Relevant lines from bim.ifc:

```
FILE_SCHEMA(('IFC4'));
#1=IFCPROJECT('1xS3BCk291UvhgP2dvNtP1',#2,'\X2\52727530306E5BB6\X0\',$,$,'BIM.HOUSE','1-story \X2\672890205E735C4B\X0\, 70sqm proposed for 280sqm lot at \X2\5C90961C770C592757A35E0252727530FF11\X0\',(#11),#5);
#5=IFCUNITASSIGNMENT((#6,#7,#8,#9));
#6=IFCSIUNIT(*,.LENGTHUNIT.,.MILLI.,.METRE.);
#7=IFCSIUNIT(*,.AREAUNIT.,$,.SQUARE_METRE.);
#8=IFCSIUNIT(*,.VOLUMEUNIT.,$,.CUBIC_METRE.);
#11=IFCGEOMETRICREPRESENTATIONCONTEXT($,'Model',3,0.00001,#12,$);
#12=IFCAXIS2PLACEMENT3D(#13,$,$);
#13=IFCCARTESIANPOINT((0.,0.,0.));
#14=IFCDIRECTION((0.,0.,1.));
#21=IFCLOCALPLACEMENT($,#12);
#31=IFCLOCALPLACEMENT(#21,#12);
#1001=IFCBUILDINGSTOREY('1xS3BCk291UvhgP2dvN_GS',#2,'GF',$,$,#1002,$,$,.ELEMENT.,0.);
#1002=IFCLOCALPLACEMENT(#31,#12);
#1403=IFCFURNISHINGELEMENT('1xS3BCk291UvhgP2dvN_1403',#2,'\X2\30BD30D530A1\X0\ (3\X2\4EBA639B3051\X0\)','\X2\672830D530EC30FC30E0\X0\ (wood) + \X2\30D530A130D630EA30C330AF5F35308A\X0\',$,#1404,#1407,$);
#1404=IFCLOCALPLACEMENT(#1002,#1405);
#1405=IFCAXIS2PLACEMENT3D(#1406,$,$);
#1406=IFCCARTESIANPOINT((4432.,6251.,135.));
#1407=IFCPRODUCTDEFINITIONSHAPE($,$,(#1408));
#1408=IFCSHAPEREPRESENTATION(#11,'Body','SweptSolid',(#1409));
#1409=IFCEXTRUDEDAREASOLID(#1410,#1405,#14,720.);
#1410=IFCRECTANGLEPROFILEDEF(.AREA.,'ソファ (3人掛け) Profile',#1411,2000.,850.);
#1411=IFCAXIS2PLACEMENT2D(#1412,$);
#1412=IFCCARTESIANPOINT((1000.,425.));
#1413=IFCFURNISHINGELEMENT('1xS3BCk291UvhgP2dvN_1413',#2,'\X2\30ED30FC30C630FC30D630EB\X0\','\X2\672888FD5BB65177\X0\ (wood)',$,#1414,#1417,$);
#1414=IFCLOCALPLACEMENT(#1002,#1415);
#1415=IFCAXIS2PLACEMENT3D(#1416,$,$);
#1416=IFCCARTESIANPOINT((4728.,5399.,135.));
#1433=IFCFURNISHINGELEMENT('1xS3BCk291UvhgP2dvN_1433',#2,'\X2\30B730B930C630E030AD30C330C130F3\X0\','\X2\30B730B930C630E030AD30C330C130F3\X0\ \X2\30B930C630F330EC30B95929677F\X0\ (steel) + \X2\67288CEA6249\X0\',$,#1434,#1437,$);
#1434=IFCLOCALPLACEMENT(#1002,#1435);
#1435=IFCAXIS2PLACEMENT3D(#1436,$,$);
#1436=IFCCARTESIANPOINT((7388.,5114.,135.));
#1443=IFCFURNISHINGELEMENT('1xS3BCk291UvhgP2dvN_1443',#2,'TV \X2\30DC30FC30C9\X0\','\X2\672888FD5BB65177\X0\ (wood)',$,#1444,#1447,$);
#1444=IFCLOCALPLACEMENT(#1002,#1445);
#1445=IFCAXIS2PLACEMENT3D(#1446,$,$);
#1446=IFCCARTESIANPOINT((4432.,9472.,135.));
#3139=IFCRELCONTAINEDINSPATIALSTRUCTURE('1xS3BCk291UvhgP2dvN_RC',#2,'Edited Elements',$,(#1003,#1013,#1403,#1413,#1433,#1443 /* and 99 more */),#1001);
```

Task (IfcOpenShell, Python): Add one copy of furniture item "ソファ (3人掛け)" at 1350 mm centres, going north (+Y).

```python
import numpy as np
import ifcopenshell
import ifcopenshell.api.geometry
import ifcopenshell.api.root
import ifcopenshell.util.element
import ifcopenshell.util.placement

model = ifcopenshell.open("bim.ifc")


def reuse_history(source, copy):
    """copy_class also copies each property set's owner history, people and application; keep the originals."""
    for rel in copy.IsDefinedBy:
        if rel.is_a("IfcRelDefinesByProperties") and (history := rel.RelatingPropertyDefinition.OwnerHistory):
            rel.RelatingPropertyDefinition.OwnerHistory = source.OwnerHistory
            ifcopenshell.util.element.remove_deep2(model, history)


source = model.by_guid("1xS3BCk291UvhgP2dvN_1403")
base = ifcopenshell.util.placement.get_local_placement(source.ObjectPlacement)
step = np.array([0.0, 1.0, 0.0]) * 1350.0

for i in range(1, 2):
    copy = ifcopenshell.api.root.copy_class(model, product=source)
    copy.Representation = ifcopenshell.util.element.copy_deep(
        model, source.Representation, exclude=["IfcGeometricRepresentationContext", "IfcRepresentationMap"]
    )
    reuse_history(source, copy)
    matrix = base.copy()
    matrix[:3, 3] += i * step
    print("added at", matrix[:3, 3].round(3) + 0.0)
    ifcopenshell.api.geometry.edit_object_placement(model, product=copy, matrix=matrix, is_si=False)

model.write("bim_edited.ifc")
```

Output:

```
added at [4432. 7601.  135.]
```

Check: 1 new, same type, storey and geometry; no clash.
